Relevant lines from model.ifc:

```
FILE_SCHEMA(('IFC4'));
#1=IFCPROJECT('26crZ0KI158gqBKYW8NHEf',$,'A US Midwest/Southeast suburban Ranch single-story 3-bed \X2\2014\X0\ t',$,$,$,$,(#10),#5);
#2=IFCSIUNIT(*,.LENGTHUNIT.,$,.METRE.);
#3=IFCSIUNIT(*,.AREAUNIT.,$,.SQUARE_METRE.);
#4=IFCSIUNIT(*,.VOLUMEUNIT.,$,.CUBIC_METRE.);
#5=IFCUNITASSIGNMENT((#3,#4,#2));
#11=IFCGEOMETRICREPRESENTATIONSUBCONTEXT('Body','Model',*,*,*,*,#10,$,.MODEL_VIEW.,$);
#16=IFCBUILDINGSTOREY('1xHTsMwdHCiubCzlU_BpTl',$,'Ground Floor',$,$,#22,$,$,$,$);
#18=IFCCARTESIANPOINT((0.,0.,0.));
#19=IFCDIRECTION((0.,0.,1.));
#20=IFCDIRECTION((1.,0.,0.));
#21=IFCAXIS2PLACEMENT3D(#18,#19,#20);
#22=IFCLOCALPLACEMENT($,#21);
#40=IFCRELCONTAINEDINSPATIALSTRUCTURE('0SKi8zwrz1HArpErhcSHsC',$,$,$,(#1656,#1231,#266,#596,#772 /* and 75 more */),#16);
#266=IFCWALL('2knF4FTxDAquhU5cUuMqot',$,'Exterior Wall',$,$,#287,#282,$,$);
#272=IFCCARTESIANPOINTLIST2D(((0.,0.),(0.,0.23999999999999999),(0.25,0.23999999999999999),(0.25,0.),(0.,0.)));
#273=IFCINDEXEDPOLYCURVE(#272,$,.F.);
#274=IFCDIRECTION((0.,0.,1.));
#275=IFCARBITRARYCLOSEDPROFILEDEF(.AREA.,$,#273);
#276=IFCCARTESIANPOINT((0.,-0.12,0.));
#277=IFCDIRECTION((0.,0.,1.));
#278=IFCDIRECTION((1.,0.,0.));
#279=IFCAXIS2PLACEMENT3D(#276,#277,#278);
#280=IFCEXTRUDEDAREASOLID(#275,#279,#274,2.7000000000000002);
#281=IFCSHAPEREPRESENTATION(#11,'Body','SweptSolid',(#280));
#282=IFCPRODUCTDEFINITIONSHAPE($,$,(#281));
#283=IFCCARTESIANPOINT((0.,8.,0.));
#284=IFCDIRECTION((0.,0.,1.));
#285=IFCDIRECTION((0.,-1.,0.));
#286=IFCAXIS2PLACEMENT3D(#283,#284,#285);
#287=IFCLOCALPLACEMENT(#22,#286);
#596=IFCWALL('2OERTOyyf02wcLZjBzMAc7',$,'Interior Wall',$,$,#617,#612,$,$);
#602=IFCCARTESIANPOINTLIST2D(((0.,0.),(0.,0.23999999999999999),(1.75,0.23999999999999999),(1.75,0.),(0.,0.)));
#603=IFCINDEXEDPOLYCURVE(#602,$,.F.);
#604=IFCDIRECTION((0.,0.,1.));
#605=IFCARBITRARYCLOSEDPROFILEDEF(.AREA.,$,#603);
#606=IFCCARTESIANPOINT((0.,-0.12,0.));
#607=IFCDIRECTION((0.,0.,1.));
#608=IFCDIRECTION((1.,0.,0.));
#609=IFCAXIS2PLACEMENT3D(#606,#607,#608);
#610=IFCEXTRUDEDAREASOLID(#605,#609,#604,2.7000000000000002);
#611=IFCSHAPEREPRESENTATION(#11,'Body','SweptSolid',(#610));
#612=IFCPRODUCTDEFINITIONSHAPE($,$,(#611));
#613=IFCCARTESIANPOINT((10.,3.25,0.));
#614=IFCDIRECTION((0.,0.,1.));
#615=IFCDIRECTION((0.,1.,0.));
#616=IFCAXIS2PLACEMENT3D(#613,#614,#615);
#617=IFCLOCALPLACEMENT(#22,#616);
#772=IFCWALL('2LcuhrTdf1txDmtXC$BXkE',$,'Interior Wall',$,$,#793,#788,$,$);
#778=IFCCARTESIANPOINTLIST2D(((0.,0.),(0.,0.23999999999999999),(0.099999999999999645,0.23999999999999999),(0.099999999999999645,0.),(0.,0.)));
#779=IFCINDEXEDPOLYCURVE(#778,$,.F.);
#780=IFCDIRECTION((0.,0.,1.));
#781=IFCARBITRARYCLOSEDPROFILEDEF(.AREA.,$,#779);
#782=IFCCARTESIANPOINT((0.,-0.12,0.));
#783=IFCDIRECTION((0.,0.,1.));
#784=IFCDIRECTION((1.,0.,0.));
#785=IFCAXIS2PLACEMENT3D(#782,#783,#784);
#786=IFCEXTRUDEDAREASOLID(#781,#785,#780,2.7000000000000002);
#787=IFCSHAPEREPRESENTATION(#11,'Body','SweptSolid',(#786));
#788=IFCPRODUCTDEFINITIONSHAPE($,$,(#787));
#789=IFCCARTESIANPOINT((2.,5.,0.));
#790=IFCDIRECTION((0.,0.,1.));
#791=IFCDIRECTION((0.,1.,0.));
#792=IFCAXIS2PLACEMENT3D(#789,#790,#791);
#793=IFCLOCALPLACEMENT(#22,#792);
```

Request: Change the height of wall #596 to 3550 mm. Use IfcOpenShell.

```python
import ifcopenshell
import ifcopenshell.geom
import ifcopenshell.util.representation
import ifcopenshell.util.shape
import ifcopenshell.util.unit

model = ifcopenshell.open("model.ifc")
unit_scale = ifcopenshell.util.unit.calculate_unit_scale(model)
settings = ifcopenshell.geom.settings()


def volume(element):
    """Net volume in cubic metres, openings subtracted."""
    shape = ifcopenshell.geom.create_shape(settings, element)
    return ifcopenshell.util.shape.get_volume(shape.geometry)


wall = model.by_guid("2OERTOyyf02wcLZjBzMAc7")
before = volume(wall)

body = ifcopenshell.util.representation.get_representation(wall, "Model", "Body")
solid = body.Items[0]
old_height = solid.Depth
solid.Depth = 3.55 / unit_scale
after = volume(wall)

print(f"height {old_height:g} -> {solid.Depth:g}, volume {before:.3f} -> {after:.3f} m3")

model.write("model-out.ifc")
```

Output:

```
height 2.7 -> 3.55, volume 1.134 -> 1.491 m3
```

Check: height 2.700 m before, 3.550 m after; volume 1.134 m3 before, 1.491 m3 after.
